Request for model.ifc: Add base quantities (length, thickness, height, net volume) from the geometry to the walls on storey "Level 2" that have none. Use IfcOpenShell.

First a look at what the model holds.

```python
import ifcopenshell
import ifcopenshell.util.element
import ifcopenshell.util.unit

model = ifcopenshell.open("model.ifc")
print(model.schema)
for unit_type in ("LENGTHUNIT", "AREAUNIT", "VOLUMEUNIT"):
    print(unit_type, ifcopenshell.util.unit.calculate_unit_scale(model, unit_type))
storey = next(s for s in model.by_type("IfcBuildingStorey") if s.Name == "Level 2")
walls = [e for e in ifcopenshell.util.element.get_decomposition(storey) if e.is_a("IfcWall")]
for e in sorted(walls, key=lambda e: e.id()):
    print(e.id(), e.is_a(), e.Name, list(ifcopenshell.util.element.get_psets(e, qtos_only=True)), sep=" | ")
```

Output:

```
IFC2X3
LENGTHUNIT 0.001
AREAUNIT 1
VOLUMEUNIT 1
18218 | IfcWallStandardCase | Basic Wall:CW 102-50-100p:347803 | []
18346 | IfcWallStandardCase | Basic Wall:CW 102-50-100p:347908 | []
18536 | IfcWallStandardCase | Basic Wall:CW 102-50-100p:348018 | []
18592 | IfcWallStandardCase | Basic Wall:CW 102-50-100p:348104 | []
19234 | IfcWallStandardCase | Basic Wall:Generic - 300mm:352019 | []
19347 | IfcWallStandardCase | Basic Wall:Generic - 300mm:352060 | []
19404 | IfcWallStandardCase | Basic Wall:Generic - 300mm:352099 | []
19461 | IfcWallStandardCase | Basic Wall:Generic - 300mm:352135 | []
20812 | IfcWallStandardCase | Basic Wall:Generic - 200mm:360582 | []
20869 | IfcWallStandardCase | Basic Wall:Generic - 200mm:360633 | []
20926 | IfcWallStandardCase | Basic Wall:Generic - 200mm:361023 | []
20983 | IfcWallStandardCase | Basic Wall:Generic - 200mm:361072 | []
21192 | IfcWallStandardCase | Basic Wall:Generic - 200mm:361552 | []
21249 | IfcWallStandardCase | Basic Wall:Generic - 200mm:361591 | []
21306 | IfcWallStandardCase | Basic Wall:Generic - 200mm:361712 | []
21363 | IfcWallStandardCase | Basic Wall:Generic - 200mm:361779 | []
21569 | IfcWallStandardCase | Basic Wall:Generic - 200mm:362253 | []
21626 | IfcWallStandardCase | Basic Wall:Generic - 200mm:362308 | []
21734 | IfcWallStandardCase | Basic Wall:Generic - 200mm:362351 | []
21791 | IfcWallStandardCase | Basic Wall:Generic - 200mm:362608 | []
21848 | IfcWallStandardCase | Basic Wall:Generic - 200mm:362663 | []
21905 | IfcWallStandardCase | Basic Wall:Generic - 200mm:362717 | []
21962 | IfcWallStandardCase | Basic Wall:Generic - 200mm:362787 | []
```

```python
import ifcopenshell
import ifcopenshell.api.pset
import ifcopenshell.geom
import ifcopenshell.util.element
import ifcopenshell.util.shape
import ifcopenshell.util.unit

model = ifcopenshell.open("model.ifc")
unit_scale = ifcopenshell.util.unit.calculate_unit_scale(model)
volume_scale = ifcopenshell.util.unit.calculate_unit_scale(model, "VOLUMEUNIT")
settings = ifcopenshell.geom.settings()

storey = next(s for s in model.by_type("IfcBuildingStorey") if s.Name == "Level 2")
walls = [e for e in ifcopenshell.util.element.get_decomposition(storey) if e.is_a("IfcWall")]

for e in sorted(walls, key=lambda e: e.id()):
    if ifcopenshell.util.element.get_psets(e, qtos_only=True, should_inherit=False):
        continue
    # Geometry comes back in metres, in the element's own axes.
    shape = ifcopenshell.geom.create_shape(settings, e)
    values = {
        "Length": ifcopenshell.util.shape.get_x(shape.geometry) / unit_scale,
        "Width": ifcopenshell.util.shape.get_y(shape.geometry) / unit_scale,
        "Height": ifcopenshell.util.shape.get_z(shape.geometry) / unit_scale,
        "NetVolume": ifcopenshell.util.shape.get_volume(shape.geometry) / volume_scale,
    }
    qto = ifcopenshell.api.pset.add_qto(model, product=e, name="BaseQuantities")
    ifcopenshell.api.pset.edit_qto(model, qto=qto, properties=values)
    print(e.id(), {k: round(v, 3) for k, v in values.items()})

model.write("model_v2.ifc")
```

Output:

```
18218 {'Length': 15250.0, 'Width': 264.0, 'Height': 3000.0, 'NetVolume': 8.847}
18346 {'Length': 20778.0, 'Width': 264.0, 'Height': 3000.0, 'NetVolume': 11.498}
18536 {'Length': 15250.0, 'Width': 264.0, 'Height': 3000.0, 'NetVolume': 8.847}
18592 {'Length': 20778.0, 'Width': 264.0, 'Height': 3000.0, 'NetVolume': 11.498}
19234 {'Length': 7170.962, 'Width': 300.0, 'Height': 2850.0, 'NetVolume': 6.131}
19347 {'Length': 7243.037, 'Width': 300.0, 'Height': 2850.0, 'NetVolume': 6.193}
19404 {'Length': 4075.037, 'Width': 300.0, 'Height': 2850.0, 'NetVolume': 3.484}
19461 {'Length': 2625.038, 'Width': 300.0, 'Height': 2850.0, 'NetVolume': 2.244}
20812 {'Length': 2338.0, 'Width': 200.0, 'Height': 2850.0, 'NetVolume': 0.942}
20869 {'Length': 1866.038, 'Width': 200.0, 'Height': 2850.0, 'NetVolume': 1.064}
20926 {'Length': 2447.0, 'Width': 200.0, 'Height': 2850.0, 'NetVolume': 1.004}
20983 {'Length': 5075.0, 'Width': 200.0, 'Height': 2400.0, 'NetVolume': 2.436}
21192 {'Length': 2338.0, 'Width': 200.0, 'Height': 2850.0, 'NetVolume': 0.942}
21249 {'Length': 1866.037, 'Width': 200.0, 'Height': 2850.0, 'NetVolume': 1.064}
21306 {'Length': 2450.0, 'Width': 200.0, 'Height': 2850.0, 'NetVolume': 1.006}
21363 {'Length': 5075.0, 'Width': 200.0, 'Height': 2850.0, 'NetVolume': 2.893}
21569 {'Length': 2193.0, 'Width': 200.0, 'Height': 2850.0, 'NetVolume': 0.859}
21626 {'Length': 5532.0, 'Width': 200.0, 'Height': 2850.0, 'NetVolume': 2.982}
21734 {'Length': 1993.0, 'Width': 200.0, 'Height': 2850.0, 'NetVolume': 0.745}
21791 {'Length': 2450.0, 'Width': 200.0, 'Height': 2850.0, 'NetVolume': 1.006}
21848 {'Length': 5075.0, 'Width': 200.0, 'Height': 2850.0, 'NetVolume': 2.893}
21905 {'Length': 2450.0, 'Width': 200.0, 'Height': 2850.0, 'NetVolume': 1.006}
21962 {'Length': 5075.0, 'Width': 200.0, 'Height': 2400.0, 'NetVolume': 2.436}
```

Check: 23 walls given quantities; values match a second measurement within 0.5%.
